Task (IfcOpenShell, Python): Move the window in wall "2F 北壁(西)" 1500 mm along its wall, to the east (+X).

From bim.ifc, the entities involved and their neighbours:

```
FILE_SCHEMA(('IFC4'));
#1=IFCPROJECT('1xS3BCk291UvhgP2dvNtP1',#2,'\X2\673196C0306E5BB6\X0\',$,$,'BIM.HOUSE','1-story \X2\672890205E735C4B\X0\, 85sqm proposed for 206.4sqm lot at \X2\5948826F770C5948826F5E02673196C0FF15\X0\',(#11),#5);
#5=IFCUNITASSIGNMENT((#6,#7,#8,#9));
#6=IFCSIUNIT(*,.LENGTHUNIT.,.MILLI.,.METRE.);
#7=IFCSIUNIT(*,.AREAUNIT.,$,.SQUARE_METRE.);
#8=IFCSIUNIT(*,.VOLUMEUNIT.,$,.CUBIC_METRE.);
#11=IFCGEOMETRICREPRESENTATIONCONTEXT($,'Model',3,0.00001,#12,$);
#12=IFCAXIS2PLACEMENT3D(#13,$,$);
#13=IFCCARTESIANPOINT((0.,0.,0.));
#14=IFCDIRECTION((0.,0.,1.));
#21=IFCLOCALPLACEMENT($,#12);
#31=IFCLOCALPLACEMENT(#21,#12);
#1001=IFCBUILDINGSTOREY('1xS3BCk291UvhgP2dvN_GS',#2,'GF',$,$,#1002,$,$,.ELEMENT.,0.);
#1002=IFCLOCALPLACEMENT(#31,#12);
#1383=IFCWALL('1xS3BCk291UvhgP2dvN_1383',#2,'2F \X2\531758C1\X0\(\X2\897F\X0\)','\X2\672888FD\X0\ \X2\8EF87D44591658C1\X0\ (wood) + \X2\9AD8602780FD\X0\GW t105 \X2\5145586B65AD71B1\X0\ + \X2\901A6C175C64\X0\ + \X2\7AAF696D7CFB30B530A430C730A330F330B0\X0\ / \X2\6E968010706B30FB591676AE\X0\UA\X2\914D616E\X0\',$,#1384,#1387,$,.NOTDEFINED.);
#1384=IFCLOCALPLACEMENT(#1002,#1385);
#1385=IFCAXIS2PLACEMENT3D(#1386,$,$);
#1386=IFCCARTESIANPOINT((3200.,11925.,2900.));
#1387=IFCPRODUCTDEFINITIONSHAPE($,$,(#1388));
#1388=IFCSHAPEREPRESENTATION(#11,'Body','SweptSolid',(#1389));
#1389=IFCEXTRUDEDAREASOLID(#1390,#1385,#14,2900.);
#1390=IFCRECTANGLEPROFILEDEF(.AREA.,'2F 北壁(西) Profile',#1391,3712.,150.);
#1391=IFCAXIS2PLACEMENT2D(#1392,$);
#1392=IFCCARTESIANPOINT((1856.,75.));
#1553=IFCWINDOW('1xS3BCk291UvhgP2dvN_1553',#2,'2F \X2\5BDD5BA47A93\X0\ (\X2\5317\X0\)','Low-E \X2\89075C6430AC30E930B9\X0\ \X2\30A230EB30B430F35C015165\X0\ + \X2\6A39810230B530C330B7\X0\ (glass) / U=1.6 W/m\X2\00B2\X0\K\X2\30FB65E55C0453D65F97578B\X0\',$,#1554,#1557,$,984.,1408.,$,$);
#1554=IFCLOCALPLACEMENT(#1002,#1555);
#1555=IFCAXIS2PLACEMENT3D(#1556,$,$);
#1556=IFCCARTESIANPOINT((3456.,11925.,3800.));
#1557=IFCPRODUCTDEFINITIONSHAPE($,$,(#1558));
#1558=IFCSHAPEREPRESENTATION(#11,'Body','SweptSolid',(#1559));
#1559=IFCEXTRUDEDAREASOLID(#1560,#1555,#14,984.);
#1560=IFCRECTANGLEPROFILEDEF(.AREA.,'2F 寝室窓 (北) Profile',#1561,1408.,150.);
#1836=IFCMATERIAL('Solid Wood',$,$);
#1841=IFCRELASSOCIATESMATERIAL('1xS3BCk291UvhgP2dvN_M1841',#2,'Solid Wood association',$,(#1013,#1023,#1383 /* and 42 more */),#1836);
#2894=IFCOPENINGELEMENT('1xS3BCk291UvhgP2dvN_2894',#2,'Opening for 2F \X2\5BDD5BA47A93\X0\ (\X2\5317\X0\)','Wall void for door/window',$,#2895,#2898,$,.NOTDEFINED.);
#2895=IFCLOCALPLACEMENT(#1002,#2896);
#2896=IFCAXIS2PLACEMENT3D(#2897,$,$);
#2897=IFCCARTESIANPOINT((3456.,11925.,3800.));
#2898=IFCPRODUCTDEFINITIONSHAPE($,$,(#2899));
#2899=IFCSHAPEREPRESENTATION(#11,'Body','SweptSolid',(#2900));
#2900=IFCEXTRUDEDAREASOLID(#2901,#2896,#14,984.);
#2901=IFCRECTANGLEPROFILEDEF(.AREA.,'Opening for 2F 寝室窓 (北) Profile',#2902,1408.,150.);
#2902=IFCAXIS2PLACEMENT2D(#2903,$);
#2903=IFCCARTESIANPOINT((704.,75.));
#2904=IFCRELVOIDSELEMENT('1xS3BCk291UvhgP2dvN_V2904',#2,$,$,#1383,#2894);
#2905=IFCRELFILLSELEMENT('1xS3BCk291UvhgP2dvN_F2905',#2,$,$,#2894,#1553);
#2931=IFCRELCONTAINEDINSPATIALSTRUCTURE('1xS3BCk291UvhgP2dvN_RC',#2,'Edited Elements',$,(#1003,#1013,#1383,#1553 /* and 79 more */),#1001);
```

```python
import ifcopenshell
import ifcopenshell.api.geometry
import ifcopenshell.util.placement
import ifcopenshell.util.unit

model = ifcopenshell.open("bim.ifc")
unit_scale = ifcopenshell.util.unit.calculate_unit_scale(model)

window = model.by_id(1553)
opening = window.FillsVoids[0].RelatingOpeningElement
wall = opening.VoidsElements[0].RelatingBuildingElement

wall_matrix = ifcopenshell.util.placement.get_local_placement(wall.ObjectPlacement)
shift = wall_matrix[:3, 0] * 1.5 / unit_scale
before = ifcopenshell.util.placement.get_local_placement(window.ObjectPlacement)[:3, 3].copy()

# The window is not placed relative to its opening, so move both.
for product in (opening, window):
    matrix = ifcopenshell.util.placement.get_local_placement(product.ObjectPlacement)
    matrix[:3, 3] += shift
    ifcopenshell.api.geometry.edit_object_placement(model, product=product, matrix=matrix, is_si=False)

after = ifcopenshell.util.placement.get_local_placement(window.ObjectPlacement)[:3, 3]
print("window moved by", (after - before).round(3) + 0.0)

model.write("bim_edited.ifc")
```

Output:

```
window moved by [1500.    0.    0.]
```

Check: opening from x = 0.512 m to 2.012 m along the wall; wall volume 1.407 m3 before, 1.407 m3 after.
